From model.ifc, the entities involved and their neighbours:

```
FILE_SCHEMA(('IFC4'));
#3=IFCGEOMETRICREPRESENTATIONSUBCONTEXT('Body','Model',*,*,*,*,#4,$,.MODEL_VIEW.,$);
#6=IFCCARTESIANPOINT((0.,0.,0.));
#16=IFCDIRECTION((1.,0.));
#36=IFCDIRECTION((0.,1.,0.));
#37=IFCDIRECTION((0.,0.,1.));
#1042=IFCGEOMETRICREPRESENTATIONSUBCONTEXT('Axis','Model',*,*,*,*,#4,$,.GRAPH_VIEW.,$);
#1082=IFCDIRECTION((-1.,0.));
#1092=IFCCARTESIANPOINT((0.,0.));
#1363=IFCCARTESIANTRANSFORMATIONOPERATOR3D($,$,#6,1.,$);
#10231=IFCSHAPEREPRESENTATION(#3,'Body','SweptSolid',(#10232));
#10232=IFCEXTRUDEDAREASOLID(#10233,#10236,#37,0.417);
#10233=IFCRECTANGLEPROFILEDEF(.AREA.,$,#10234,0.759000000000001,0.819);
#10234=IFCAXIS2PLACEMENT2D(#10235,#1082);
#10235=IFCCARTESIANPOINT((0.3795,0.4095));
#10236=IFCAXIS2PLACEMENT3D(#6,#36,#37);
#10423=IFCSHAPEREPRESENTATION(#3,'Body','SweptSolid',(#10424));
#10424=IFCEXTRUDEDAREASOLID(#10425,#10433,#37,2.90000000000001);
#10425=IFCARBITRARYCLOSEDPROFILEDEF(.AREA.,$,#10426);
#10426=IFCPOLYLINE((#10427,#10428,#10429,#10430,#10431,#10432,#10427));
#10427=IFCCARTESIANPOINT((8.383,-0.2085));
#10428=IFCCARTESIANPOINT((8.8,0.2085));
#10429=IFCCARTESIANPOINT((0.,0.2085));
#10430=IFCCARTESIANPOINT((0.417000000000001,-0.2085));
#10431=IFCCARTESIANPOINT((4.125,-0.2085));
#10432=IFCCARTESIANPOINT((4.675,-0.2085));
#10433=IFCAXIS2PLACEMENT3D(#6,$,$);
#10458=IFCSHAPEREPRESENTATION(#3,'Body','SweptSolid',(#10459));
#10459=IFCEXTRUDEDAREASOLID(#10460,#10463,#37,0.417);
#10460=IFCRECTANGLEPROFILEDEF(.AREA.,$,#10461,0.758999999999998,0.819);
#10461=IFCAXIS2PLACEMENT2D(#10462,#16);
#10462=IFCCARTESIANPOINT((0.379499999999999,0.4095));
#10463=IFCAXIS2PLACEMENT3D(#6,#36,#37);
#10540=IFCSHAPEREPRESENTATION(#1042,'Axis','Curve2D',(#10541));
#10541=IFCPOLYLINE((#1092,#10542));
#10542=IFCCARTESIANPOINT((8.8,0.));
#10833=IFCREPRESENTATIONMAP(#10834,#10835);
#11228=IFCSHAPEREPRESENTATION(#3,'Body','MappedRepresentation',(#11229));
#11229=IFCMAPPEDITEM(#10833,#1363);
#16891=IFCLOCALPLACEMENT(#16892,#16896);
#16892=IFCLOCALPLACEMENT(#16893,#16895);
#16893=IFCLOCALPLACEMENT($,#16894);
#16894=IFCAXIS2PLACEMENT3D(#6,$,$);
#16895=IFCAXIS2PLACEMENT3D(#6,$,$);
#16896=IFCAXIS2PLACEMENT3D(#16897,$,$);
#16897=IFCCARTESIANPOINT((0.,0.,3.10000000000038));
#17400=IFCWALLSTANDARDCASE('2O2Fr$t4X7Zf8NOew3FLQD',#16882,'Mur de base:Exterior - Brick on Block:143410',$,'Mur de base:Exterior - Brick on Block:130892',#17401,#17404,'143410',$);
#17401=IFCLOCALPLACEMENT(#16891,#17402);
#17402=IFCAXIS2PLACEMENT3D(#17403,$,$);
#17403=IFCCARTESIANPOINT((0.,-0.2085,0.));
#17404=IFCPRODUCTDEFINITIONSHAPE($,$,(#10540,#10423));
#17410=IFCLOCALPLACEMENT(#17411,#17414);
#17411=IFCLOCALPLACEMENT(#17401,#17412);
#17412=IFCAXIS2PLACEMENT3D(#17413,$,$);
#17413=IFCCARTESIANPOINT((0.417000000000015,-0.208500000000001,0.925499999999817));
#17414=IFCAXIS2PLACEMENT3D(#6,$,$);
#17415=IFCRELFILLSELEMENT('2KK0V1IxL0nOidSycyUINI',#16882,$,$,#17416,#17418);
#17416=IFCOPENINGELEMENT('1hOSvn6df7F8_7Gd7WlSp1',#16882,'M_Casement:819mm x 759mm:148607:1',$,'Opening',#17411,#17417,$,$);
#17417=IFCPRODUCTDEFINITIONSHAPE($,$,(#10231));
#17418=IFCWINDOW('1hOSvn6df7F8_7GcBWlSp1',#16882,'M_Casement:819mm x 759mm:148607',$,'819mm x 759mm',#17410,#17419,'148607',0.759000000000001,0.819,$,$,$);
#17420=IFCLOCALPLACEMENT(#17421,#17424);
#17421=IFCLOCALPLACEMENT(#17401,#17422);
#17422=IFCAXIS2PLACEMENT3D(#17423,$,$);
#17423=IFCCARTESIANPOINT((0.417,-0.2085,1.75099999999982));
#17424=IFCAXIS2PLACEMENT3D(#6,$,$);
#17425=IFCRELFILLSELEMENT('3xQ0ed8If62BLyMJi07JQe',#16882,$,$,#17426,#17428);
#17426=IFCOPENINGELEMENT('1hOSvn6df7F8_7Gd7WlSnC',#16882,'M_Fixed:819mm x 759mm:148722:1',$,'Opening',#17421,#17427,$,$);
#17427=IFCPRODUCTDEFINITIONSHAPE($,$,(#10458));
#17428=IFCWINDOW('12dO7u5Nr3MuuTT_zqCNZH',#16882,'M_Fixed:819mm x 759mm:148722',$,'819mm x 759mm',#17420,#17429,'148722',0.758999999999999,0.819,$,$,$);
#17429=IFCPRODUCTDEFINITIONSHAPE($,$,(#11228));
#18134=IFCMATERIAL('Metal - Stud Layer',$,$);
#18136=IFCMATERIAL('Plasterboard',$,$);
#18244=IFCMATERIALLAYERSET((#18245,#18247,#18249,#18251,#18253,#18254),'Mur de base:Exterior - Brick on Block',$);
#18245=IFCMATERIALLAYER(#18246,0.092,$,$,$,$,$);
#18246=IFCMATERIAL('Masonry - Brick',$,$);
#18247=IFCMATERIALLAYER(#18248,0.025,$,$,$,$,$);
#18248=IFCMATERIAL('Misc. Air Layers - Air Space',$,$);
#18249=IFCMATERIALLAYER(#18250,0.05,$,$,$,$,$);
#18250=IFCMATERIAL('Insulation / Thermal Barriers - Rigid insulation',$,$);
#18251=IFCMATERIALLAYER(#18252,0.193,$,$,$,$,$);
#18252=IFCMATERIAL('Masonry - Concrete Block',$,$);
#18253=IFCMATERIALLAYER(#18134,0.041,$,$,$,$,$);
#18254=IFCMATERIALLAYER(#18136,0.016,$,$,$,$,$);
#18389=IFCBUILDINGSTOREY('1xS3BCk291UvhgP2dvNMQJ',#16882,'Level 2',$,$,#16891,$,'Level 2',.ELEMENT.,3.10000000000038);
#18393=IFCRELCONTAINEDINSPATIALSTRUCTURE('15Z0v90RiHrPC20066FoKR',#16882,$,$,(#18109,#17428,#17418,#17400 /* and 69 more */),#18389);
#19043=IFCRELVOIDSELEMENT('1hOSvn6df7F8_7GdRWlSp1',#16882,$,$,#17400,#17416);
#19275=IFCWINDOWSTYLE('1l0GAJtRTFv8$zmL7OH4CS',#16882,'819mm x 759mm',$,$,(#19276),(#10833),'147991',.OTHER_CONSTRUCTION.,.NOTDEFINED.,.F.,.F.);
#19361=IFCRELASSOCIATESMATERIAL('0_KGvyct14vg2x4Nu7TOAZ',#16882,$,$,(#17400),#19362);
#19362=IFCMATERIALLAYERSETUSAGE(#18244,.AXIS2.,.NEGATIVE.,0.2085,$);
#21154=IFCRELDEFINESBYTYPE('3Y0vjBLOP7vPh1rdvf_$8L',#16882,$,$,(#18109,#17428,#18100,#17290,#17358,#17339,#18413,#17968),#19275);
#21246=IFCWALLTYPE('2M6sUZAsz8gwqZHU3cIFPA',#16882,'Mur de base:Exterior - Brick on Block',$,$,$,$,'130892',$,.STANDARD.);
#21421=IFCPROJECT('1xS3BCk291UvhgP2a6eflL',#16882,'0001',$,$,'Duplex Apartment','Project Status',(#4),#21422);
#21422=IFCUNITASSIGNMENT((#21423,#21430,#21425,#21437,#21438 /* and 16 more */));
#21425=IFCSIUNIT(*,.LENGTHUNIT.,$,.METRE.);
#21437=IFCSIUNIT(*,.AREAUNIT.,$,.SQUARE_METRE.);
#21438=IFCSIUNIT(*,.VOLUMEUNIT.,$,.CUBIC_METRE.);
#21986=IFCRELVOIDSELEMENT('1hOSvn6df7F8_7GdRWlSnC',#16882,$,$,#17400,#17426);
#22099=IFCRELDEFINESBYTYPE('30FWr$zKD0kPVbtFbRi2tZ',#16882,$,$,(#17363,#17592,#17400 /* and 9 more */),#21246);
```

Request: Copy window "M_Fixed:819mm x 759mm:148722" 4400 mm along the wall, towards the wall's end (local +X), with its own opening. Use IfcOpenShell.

```python
import ifcopenshell
import ifcopenshell.api.feature
import ifcopenshell.api.geometry
import ifcopenshell.api.root
import ifcopenshell.geom
import ifcopenshell.util.element
import ifcopenshell.util.placement
import ifcopenshell.util.shape

model = ifcopenshell.open("model.ifc")
settings = ifcopenshell.geom.settings()


def volume(element):
    """Net volume in cubic metres, openings subtracted."""
    shape = ifcopenshell.geom.create_shape(settings, element)
    return ifcopenshell.util.shape.get_volume(shape.geometry)


def reuse_history(source, copy):
    """copy_class also copies each property set's owner history, people and application; keep the originals."""
    for rel in copy.IsDefinedBy:
        if rel.is_a("IfcRelDefinesByProperties") and (history := rel.RelatingPropertyDefinition.OwnerHistory):
            rel.RelatingPropertyDefinition.OwnerHistory = source.OwnerHistory
            ifcopenshell.util.element.remove_deep2(model, history)


window = model.by_guid("12dO7u5Nr3MuuTT_zqCNZH")
opening = window.FillsVoids[0].RelatingOpeningElement
wall = opening.VoidsElements[0].RelatingBuildingElement
before = volume(wall)
shift = ifcopenshell.util.placement.get_local_placement(wall.ObjectPlacement)[:3, 0] * 4.4

# copy_class copies the void relationship, type, container and properties, but no geometry.
new_opening = ifcopenshell.api.root.copy_class(model, product=opening)
new_opening.Representation = ifcopenshell.util.element.copy_deep(
    model, opening.Representation, exclude=["IfcGeometricRepresentationContext", "IfcRepresentationMap"]
)
new_opening.Name = "M_Fixed:819mm x 759mm"
new_window = ifcopenshell.api.root.copy_class(model, product=window)
new_window.Representation = ifcopenshell.util.element.copy_deep(
    model, window.Representation, exclude=["IfcGeometricRepresentationContext", "IfcRepresentationMap"]
)
new_window.Name = "M_Fixed:819mm x 759mm"
new_window.Tag = None
reuse_history(window, new_window)
ifcopenshell.api.feature.add_filling(model, opening=new_opening, element=new_window)

for old, new in ((opening, new_opening), (window, new_window)):
    matrix = ifcopenshell.util.placement.get_local_placement(old.ObjectPlacement)
    matrix[:3, 3] += shift
    ifcopenshell.api.geometry.edit_object_placement(model, product=new, matrix=matrix, is_si=False)

after = volume(wall)

print(f"wall volume {before:.3f} -> {after:.3f} m3")

model.write("model_rev.ifc")
```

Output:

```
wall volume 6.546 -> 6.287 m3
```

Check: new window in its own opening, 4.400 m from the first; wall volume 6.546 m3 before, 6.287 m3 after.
